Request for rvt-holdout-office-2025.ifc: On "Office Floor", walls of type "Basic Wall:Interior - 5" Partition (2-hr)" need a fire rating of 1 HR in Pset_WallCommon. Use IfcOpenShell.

First a look at what the model holds.

```python
import ifcopenshell
import ifcopenshell.util.element

model = ifcopenshell.open("rvt-holdout-office-2025.ifc")
print(model.schema)
storey = next(s for s in model.by_type("IfcBuildingStorey") if s.Name == "Office Floor")
walls = [e for e in ifcopenshell.util.element.get_decomposition(storey) if e.is_a("IfcWall")]
seen = {}
for e in walls:
    element_type = ifcopenshell.util.element.get_type(e)
    key = (element_type.Name if element_type != e and element_type else None, ifcopenshell.util.element.get_pset(e, "Pset_WallCommon", "FireRating"))
    seen[key] = seen.get(key, 0) + 1
for (name, value), count in sorted(seen.items(), key=str):
    print(count, "x", name, "|", value)
```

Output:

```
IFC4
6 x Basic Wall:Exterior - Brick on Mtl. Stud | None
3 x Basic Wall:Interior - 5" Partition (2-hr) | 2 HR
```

```python
import ifcopenshell
import ifcopenshell.api.pset
import ifcopenshell.util.element

model = ifcopenshell.open("rvt-holdout-office-2025.ifc")

storey = next(s for s in model.by_type("IfcBuildingStorey") if s.Name == "Office Floor")
walls = [e for e in ifcopenshell.util.element.get_decomposition(storey) if e.is_a("IfcWall")]

count = 0
for e in walls:
    element_type = ifcopenshell.util.element.get_type(e)
    if element_type in (None, e) or element_type.Name != 'Basic Wall:Interior - 5" Partition (2-hr)':
        continue
    # add_pset returns the element's existing set when there is one.
    pset = ifcopenshell.api.pset.add_pset(model, product=e, name="Pset_WallCommon")
    ifcopenshell.api.pset.edit_pset(model, pset=pset, properties={"FireRating": "1 HR"})
    count += 1

print(count, "walls updated")

model.write("rvt-holdout-office-2025_updated.ifc")
```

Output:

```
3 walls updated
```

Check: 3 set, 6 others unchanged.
